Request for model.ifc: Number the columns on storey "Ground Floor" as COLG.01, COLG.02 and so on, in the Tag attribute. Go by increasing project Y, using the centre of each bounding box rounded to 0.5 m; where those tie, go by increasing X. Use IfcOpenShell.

First a look at what the model holds.

```python
import ifcopenshell
import ifcopenshell.util.element
import ifcopenshell.util.placement

model = ifcopenshell.open("model.ifc")
print(model.schema)
storey = next(s for s in model.by_type("IfcBuildingStorey") if s.Name == "Ground Floor")
columns = [e for e in ifcopenshell.util.element.get_decomposition(storey) if e.is_a("IfcColumn")]
for e in sorted(columns, key=lambda e: e.id()):
    origin = ifcopenshell.util.placement.get_local_placement(e.ObjectPlacement)[:3, 3]
    print(e.id(), e.Tag, e.Name, origin.round(2) + 0.0, sep=" | ")
```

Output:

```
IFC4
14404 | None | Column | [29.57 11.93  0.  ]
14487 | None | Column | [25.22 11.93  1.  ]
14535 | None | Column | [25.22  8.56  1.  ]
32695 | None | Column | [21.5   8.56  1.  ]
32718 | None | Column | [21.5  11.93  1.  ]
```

```python
import ifcopenshell
import ifcopenshell.geom
import ifcopenshell.util.element
import ifcopenshell.util.shape

model = ifcopenshell.open("model.ifc")
settings = ifcopenshell.geom.settings()
settings.set("use-world-coords", True)


def centre(element):
    shape = ifcopenshell.geom.create_shape(settings, element)
    return ifcopenshell.util.shape.get_bbox_centroid(shape.geometry)


storey = next(s for s in model.by_type("IfcBuildingStorey") if s.Name == "Ground Floor")
columns = [e for e in ifcopenshell.util.element.get_decomposition(storey) if e.is_a("IfcColumn")]

# Insertion points can sit at a corner or the storey origin, so sort by the geometry (in metres).
centres = {e: centre(e) for e in columns}
columns.sort(key=lambda e: (round(centres[e][1] / 0.5), centres[e][0]))

for i, e in enumerate(columns, start=1):
    number = f"COLG.{i:02d}"
    e.Tag = number
    print(e.id(), number)

model.write("model_edited.ifc")
```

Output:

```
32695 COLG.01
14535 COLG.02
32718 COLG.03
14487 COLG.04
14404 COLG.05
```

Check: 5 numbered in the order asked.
